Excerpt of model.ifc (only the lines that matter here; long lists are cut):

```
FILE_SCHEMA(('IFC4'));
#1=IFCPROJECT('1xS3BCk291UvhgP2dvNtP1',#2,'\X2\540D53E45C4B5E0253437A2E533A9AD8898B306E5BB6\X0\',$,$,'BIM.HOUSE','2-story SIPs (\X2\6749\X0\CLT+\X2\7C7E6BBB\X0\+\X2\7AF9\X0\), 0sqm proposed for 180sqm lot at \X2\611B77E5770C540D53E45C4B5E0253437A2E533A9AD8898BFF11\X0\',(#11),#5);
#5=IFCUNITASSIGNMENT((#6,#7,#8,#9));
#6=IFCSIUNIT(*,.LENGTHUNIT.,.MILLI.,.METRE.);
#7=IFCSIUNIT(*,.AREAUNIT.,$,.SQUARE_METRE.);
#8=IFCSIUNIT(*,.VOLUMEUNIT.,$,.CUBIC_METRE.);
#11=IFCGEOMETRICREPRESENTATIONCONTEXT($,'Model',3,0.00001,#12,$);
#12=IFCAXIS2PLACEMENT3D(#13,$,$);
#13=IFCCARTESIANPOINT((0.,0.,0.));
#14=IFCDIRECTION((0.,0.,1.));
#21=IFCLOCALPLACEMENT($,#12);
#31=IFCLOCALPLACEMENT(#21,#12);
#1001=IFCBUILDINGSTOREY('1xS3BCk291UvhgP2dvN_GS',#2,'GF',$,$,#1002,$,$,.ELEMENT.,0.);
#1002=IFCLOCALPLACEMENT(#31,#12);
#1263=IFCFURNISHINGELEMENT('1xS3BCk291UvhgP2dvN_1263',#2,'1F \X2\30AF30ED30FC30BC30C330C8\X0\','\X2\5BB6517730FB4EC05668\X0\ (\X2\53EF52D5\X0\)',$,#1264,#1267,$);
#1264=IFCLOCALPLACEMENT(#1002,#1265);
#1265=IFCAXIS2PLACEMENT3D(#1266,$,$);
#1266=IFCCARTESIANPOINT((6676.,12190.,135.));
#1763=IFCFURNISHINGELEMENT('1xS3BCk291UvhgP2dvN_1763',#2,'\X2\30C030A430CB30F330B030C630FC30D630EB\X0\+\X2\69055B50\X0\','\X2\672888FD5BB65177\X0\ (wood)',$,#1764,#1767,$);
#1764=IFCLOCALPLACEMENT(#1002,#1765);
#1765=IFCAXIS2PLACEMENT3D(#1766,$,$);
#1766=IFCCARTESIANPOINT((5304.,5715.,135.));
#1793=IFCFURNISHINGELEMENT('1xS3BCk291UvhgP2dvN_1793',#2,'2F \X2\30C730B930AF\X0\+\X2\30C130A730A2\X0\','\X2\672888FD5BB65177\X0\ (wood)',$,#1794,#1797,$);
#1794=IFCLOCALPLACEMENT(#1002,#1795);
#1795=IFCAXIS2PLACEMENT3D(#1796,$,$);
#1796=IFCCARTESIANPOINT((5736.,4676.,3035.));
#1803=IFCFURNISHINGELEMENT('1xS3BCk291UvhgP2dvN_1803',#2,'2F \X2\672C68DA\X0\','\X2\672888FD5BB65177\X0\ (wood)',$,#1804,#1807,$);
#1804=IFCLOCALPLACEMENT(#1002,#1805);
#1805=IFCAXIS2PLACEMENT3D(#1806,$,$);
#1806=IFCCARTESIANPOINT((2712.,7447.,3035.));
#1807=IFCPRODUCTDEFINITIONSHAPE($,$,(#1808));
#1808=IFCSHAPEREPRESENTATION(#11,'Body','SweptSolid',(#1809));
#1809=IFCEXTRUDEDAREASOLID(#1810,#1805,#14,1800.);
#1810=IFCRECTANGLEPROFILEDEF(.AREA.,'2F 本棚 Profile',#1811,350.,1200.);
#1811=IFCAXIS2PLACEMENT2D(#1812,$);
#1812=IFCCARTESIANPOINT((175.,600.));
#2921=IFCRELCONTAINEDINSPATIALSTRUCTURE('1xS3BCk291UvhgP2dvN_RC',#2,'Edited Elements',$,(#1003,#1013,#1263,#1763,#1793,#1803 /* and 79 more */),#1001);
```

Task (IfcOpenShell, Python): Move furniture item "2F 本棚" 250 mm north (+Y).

```python
import ifcopenshell
import ifcopenshell.api.geometry
import ifcopenshell.util.placement

model = ifcopenshell.open("model.ifc")

item = model.by_guid("1xS3BCk291UvhgP2dvN_1803")
matrix = ifcopenshell.util.placement.get_local_placement(item.ObjectPlacement)
matrix[1, 3] += 250.0
ifcopenshell.api.geometry.edit_object_placement(model, product=item, matrix=matrix, is_si=False)

print(ifcopenshell.util.placement.get_local_placement(item.ObjectPlacement).round(3) + 0.0)

model.write("model_edited.ifc")
```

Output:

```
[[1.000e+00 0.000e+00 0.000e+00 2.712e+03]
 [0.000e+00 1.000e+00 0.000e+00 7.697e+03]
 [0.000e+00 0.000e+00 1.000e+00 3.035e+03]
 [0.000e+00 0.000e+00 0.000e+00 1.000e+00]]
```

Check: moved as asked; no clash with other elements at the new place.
